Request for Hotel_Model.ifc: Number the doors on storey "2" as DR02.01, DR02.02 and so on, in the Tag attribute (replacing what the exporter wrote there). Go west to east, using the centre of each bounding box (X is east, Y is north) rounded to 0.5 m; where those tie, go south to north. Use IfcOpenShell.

First a look at what the model holds.

```python
import ifcopenshell
import ifcopenshell.util.element
import ifcopenshell.util.placement

model = ifcopenshell.open("Hotel_Model.ifc")
print(model.schema)
storey = next(s for s in model.by_type("IfcBuildingStorey") if s.Name == "2")
doors = [e for e in ifcopenshell.util.element.get_decomposition(storey) if e.is_a("IfcDoor")]
for e in sorted(doors, key=lambda e: e.id()):
    origin = ifcopenshell.util.placement.get_local_placement(e.ObjectPlacement)[:3, 3]
    print(e.id(), e.Tag, e.Name, origin.round(2) + 0.0, sep=" | ")
```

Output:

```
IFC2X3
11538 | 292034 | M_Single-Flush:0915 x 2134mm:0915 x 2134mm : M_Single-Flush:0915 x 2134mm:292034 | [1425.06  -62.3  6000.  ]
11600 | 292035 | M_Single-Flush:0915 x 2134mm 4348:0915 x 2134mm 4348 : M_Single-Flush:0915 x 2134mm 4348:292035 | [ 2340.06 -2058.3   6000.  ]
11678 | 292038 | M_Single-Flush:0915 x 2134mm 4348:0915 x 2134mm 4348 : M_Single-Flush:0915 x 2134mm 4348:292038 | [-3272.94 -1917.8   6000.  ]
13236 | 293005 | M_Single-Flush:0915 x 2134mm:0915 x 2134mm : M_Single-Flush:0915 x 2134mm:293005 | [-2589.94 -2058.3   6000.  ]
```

```python
import ifcopenshell
import ifcopenshell.geom
import ifcopenshell.util.element
import ifcopenshell.util.shape

model = ifcopenshell.open("Hotel_Model.ifc")
settings = ifcopenshell.geom.settings()
settings.set("use-world-coords", True)


def centre(element):
    shape = ifcopenshell.geom.create_shape(settings, element)
    return ifcopenshell.util.shape.get_bbox_centroid(shape.geometry)


storey = next(s for s in model.by_type("IfcBuildingStorey") if s.Name == "2")
doors = [e for e in ifcopenshell.util.element.get_decomposition(storey) if e.is_a("IfcDoor")]

# Insertion points can sit at a corner or the storey origin, so sort by the geometry (in metres).
centres = {e: centre(e) for e in doors}
doors.sort(key=lambda e: (round(centres[e][0] / 0.5), centres[e][1]))

for i, e in enumerate(doors, start=1):
    number = f"DR02.{i:02d}"
    e.Tag = number
    print(e.id(), number)

model.write("Hotel_Model_edited.ifc")
```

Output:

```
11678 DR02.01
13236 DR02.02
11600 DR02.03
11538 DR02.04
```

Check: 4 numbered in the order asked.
